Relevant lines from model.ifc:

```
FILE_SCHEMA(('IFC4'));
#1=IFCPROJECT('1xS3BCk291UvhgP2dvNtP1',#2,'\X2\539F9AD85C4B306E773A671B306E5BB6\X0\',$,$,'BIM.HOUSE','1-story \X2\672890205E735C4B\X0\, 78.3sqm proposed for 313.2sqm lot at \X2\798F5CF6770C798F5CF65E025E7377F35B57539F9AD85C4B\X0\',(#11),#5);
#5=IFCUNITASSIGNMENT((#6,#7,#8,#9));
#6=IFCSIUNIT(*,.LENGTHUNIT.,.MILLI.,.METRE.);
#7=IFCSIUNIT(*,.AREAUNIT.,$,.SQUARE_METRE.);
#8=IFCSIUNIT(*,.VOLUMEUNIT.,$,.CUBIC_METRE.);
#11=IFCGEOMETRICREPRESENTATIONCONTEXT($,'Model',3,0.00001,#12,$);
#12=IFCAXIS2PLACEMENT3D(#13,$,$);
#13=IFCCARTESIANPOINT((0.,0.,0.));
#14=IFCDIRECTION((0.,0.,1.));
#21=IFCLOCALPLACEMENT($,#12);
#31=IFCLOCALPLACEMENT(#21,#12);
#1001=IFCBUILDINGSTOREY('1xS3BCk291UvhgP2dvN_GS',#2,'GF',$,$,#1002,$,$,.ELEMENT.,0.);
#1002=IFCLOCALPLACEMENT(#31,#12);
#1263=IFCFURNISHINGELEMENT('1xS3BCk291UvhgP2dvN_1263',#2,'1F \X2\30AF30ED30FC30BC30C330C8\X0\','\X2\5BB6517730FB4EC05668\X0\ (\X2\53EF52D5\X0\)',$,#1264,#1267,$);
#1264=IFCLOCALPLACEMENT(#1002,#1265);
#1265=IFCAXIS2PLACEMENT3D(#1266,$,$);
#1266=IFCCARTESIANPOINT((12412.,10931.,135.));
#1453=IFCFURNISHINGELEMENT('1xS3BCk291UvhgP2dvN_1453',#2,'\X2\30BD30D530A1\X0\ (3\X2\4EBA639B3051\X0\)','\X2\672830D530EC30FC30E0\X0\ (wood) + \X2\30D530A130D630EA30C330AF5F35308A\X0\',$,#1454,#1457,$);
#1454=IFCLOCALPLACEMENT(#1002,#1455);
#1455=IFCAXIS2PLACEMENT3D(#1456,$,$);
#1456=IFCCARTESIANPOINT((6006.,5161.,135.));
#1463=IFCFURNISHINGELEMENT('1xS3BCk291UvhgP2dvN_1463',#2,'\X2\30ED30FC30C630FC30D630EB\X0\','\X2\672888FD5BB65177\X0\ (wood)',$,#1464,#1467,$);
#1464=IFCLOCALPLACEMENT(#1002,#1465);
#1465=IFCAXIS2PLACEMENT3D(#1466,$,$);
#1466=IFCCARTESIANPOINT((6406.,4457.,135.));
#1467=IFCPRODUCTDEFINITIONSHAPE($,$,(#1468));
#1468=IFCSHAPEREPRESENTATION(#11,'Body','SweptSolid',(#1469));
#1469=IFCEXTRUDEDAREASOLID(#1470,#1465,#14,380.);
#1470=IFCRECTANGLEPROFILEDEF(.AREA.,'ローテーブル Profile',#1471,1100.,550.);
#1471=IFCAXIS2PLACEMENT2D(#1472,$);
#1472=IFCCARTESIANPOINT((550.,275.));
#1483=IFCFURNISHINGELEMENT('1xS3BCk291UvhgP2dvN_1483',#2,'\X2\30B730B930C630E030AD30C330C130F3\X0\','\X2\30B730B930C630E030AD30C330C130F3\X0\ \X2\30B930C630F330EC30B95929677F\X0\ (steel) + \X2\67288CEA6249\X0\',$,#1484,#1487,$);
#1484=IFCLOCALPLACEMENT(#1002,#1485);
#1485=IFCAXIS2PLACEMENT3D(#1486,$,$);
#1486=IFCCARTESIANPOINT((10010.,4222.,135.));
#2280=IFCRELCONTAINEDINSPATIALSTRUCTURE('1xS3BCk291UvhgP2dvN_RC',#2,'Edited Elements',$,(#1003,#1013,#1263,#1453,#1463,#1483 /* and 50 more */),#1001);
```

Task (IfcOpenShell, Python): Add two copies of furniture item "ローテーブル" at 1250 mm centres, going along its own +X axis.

```python
import ifcopenshell
import ifcopenshell.api.geometry
import ifcopenshell.api.root
import ifcopenshell.util.element
import ifcopenshell.util.placement
import ifcopenshell.util.unit

model = ifcopenshell.open("model.ifc")
unit_scale = ifcopenshell.util.unit.calculate_unit_scale(model)


def reuse_history(source, copy):
    """copy_class also copies each property set's owner history, people and application; keep the originals."""
    for rel in copy.IsDefinedBy:
        if rel.is_a("IfcRelDefinesByProperties") and (history := rel.RelatingPropertyDefinition.OwnerHistory):
            rel.RelatingPropertyDefinition.OwnerHistory = source.OwnerHistory
            ifcopenshell.util.element.remove_deep2(model, history)


source = model.by_guid("1xS3BCk291UvhgP2dvN_1463")
base = ifcopenshell.util.placement.get_local_placement(source.ObjectPlacement)
step = base[:3, 0] * 1.25 / unit_scale

for i in range(1, 3):
    copy = ifcopenshell.api.root.copy_class(model, product=source)
    copy.Representation = ifcopenshell.util.element.copy_deep(
        model, source.Representation, exclude=["IfcGeometricRepresentationContext", "IfcRepresentationMap"]
    )
    reuse_history(source, copy)
    matrix = base.copy()
    matrix[:3, 3] += i * step
    print("added at", matrix[:3, 3].round(3) + 0.0)
    ifcopenshell.api.geometry.edit_object_placement(model, product=copy, matrix=matrix, is_si=False)

model.write("model_updated.ifc")
```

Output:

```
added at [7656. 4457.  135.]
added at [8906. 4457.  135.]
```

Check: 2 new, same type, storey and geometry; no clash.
